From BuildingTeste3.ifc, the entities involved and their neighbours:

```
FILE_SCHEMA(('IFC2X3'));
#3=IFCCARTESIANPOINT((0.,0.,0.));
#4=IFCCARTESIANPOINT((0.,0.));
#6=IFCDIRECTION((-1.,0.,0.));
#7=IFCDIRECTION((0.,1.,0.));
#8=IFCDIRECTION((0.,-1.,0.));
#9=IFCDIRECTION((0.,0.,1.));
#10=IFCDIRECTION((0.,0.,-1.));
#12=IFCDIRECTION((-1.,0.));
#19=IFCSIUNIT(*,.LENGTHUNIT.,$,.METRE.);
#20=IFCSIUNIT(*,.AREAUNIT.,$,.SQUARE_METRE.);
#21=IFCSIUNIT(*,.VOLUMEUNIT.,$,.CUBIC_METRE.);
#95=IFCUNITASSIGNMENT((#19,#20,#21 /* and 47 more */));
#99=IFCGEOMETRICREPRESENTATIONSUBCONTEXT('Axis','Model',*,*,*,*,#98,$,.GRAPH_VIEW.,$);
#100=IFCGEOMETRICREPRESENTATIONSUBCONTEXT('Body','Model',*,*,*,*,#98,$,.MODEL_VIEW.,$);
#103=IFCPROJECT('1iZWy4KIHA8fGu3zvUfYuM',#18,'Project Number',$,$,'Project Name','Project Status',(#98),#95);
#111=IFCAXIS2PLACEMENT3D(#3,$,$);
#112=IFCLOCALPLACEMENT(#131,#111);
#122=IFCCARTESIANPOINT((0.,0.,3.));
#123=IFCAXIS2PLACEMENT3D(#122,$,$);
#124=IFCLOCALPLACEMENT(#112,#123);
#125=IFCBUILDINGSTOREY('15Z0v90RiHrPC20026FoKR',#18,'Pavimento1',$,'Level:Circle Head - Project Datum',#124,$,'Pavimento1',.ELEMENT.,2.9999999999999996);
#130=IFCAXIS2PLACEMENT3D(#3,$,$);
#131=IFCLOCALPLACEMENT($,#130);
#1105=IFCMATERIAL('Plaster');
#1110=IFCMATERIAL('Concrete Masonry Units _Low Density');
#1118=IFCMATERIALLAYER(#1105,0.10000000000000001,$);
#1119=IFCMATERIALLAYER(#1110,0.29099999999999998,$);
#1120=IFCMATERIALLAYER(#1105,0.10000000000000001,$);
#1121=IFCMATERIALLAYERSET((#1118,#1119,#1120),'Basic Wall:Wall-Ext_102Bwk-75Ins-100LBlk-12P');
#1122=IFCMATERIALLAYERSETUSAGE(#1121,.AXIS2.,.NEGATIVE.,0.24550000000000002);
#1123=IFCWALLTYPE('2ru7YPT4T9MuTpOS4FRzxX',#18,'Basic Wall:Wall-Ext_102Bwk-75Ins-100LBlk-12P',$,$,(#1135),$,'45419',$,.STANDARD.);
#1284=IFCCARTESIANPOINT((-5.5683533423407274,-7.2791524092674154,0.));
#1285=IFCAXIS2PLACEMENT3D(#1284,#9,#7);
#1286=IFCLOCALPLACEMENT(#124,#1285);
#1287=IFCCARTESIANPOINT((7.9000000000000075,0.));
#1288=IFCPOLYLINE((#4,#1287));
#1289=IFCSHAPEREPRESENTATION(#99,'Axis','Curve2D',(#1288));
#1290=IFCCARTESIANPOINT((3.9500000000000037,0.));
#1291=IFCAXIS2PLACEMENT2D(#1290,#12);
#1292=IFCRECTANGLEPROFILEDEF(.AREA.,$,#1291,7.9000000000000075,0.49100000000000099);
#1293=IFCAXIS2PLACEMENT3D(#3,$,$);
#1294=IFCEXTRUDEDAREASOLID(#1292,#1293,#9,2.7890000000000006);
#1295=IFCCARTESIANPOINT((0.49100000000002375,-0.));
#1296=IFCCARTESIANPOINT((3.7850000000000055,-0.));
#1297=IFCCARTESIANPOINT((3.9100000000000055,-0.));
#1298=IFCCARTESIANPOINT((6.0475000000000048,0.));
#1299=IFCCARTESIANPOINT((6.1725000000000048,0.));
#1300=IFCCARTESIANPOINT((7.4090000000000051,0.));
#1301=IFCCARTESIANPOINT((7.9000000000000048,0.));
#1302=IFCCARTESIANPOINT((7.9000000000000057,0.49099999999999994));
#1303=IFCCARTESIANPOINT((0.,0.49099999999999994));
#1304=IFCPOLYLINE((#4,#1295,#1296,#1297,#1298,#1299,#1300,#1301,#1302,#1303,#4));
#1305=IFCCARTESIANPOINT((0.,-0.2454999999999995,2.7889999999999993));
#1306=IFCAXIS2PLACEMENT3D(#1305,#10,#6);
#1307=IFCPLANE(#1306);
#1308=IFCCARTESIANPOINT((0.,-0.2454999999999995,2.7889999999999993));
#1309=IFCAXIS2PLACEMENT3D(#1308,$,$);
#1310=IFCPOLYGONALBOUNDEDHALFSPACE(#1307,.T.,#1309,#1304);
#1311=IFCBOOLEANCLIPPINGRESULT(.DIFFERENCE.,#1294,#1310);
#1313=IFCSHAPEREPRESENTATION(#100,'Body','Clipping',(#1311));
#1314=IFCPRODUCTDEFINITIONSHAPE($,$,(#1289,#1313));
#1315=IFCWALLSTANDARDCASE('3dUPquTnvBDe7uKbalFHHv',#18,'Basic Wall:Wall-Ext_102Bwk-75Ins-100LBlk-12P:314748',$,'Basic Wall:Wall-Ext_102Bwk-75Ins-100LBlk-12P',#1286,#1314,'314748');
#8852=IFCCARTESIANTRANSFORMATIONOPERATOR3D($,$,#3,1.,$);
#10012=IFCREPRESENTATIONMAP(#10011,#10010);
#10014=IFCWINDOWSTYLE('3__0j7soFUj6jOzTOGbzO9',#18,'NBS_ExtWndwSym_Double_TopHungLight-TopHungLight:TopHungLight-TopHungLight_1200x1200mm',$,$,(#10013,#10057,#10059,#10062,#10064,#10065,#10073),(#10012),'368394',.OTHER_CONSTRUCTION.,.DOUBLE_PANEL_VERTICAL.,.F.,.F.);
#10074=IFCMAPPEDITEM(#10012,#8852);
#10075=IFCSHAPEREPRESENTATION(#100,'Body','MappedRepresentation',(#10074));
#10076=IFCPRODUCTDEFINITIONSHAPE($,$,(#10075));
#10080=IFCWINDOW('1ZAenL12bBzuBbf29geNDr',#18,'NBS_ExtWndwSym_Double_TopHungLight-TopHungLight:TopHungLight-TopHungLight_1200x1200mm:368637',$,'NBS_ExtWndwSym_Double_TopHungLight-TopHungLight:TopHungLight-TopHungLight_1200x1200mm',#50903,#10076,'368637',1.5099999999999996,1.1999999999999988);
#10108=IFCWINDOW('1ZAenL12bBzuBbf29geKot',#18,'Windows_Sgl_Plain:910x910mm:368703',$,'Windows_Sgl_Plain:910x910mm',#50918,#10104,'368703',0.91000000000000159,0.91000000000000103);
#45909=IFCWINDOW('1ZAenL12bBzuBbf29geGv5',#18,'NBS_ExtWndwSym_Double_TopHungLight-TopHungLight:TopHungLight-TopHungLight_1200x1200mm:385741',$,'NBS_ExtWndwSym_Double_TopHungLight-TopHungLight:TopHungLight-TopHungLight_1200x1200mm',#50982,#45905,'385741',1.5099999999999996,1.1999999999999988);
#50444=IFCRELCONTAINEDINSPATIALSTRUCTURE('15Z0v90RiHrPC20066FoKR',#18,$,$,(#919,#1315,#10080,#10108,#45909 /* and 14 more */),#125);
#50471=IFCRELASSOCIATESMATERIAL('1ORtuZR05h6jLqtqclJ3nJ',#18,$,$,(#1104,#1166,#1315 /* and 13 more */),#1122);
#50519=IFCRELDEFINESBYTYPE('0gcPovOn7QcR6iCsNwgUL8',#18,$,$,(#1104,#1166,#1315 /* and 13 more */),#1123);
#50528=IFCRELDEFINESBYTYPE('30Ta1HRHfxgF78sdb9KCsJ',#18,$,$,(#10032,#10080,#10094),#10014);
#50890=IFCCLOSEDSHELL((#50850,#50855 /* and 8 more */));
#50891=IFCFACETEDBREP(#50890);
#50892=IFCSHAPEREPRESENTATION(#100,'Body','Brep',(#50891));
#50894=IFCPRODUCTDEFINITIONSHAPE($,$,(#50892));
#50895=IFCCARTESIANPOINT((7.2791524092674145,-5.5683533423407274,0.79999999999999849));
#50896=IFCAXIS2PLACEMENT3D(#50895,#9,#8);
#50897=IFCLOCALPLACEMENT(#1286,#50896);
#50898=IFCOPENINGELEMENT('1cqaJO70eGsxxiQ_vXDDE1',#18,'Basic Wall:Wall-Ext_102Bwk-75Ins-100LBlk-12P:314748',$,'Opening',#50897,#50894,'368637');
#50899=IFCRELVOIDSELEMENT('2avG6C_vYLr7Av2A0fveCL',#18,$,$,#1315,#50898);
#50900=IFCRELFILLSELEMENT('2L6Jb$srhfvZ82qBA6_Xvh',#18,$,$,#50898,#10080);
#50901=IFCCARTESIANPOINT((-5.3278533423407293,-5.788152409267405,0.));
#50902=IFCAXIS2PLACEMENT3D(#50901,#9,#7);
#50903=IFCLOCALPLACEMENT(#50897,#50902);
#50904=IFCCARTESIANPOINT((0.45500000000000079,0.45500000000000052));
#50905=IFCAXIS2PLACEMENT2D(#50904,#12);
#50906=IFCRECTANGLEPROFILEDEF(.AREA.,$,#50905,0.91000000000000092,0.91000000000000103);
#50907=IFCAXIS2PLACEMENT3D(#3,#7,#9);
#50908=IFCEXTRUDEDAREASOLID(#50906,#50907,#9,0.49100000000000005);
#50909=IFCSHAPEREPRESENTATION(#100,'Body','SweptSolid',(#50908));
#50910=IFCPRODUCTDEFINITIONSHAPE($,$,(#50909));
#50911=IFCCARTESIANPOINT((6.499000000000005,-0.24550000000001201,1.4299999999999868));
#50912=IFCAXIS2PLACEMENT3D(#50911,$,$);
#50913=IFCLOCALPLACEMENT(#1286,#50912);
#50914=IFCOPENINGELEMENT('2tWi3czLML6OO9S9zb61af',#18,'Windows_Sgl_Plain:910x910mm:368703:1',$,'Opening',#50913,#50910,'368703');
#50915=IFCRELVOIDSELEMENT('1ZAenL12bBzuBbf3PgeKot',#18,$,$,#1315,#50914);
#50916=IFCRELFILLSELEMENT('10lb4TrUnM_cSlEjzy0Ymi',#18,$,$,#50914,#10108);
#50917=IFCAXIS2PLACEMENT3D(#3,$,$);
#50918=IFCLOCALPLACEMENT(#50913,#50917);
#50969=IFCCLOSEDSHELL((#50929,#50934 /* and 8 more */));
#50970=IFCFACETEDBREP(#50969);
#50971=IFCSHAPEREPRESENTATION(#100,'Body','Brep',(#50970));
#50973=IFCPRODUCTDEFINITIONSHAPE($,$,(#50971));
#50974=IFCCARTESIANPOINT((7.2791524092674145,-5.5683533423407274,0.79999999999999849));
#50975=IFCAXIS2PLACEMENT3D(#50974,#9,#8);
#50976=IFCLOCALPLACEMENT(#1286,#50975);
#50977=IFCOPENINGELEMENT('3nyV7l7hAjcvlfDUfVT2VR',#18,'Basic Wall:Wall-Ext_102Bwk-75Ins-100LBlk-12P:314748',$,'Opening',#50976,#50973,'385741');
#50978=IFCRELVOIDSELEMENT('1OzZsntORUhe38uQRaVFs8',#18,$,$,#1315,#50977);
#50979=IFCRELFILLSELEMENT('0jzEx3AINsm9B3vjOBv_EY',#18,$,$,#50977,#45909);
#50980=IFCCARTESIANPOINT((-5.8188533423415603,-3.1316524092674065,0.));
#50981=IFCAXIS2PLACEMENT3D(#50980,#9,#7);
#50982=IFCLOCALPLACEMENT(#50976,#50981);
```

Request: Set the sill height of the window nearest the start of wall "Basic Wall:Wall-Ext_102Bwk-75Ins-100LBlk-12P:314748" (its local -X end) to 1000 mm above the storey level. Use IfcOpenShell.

```python
import numpy as np
import ifcopenshell
import ifcopenshell.api.geometry
import ifcopenshell.geom
import ifcopenshell.util.element
import ifcopenshell.util.placement
import ifcopenshell.util.shape
import ifcopenshell.util.unit

model = ifcopenshell.open("BuildingTeste3.ifc")
unit_scale = ifcopenshell.util.unit.calculate_unit_scale(model)

window = model.by_guid("1ZAenL12bBzuBbf29geNDr")
opening = window.FillsVoids[0].RelatingOpeningElement
storey = ifcopenshell.util.element.get_container(window, ifc_class="IfcBuildingStorey")
level = ifcopenshell.util.placement.get_local_placement(storey.ObjectPlacement)[2, 3]

# The opening's origin need not be at the sill, so measure its lowest point.
shape = ifcopenshell.geom.create_shape(ifcopenshell.geom.settings(), opening)
bottom = ifcopenshell.util.shape.get_shape_bottom_elevation(shape, shape.geometry) / unit_scale
dz = level + 1 / unit_scale - bottom

shift = np.array([0.0, 0.0, dz])
# The window is placed relative to its opening, so it follows when the opening moves.
matrix = ifcopenshell.util.placement.get_local_placement(opening.ObjectPlacement)
matrix[:3, 3] += shift
ifcopenshell.api.geometry.edit_object_placement(
    model, product=opening, matrix=matrix, is_si=False, should_transform_children=True
)

print(f"moved by {dz * unit_scale:+.3f} m")

model.write("BuildingTeste3_edited.ifc")
```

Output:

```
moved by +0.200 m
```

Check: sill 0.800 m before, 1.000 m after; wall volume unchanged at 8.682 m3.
